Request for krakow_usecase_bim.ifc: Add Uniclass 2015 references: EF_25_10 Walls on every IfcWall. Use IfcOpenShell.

First a look at what the model holds.

```python
import ifcopenshell

model = ifcopenshell.open("krakow_usecase_bim.ifc")
print(model.schema)
print("classifications:", [c.Name for c in model.by_type("IfcClassification")])
for ifc_class in ("IfcDoor", "IfcRoof", "IfcStair", "IfcWall", "IfcWindow"):
    print(ifc_class, len(model.by_type(ifc_class)))
```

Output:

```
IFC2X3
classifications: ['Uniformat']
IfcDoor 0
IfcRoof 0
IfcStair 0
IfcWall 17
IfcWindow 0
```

```python
import ifcopenshell
import ifcopenshell.api.classification

model = ifcopenshell.open("krakow_usecase_bim.ifc")

# IFC2X3 requires Source and Edition and has no link from the project to the system.
system = model.create_entity("IfcClassification", Source="NBS", Edition="2015", Name="Uniclass 2015")

codes = {
    "IfcWall": ("EF_25_10", "Walls"),
}
for ifc_class, (code, name) in codes.items():
    products = model.by_type(ifc_class)
    ifcopenshell.api.classification.add_reference(
        model, products=products, classification=system, identification=code, name=name
    )
    print(code, len(products))

model.write("krakow_usecase_bim-out.ifc")
```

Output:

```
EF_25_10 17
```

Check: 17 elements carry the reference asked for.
